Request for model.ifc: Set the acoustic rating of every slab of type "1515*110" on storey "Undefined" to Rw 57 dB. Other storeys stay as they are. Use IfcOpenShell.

First a look at what the model holds.

```python
import ifcopenshell
import ifcopenshell.util.element

model = ifcopenshell.open("model.ifc")
print(model.schema)
storey = next(s for s in model.by_type("IfcBuildingStorey") if s.Name == "Undefined")
slabs = [e for e in ifcopenshell.util.element.get_decomposition(storey) if e.is_a("IfcSlab")]
seen = {}
for e in slabs:
    element_type = ifcopenshell.util.element.get_type(e)
    key = (element_type.Name if element_type != e and element_type else None, ifcopenshell.util.element.get_pset(e, "Pset_SlabCommon", "AcousticRating"))
    seen[key] = seen.get(key, 0) + 1
for (name, value), count in sorted(seen.items(), key=str):
    print(count, "x", name, "|", value)
```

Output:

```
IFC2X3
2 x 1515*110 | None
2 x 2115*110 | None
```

```python
import ifcopenshell
import ifcopenshell.api.pset
import ifcopenshell.util.element

model = ifcopenshell.open("model.ifc")

storey = next(s for s in model.by_type("IfcBuildingStorey") if s.Name == "Undefined")
slabs = [e for e in ifcopenshell.util.element.get_decomposition(storey) if e.is_a("IfcSlab")]

count = 0
for e in slabs:
    element_type = ifcopenshell.util.element.get_type(e)
    if element_type in (None, e) or element_type.Name != "1515*110":
        continue
    # add_pset returns the element's existing set when there is one.
    pset = ifcopenshell.api.pset.add_pset(model, product=e, name="Pset_SlabCommon")
    ifcopenshell.api.pset.edit_pset(model, pset=pset, properties={"AcousticRating": "Rw 57 dB"})
    count += 1

print(count, "slabs updated")

model.write("model-out.ifc")
```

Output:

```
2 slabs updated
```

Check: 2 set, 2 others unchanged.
